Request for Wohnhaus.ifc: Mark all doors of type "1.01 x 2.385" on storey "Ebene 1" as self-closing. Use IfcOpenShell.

First a look at what the model holds.

```python
import ifcopenshell
import ifcopenshell.util.element

model = ifcopenshell.open("Wohnhaus.ifc")
print(model.schema)
storey = next(s for s in model.by_type("IfcBuildingStorey") if s.Name == "Ebene 1")
doors = [e for e in ifcopenshell.util.element.get_decomposition(storey) if e.is_a("IfcDoor")]
seen = {}
for e in doors:
    element_type = ifcopenshell.util.element.get_type(e)
    key = (element_type.Name if element_type != e and element_type else None, ifcopenshell.util.element.get_pset(e, "Pset_DoorCommon", "SelfClosing"))
    seen[key] = seen.get(key, 0) + 1
for (name, value), count in sorted(seen.items(), key=str):
    print(count, "x", name, "|", value)
```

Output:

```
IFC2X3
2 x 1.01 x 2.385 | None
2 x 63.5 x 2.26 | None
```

```python
import ifcopenshell
import ifcopenshell.api.pset
import ifcopenshell.util.element

model = ifcopenshell.open("Wohnhaus.ifc")

storey = next(s for s in model.by_type("IfcBuildingStorey") if s.Name == "Ebene 1")
doors = [e for e in ifcopenshell.util.element.get_decomposition(storey) if e.is_a("IfcDoor")]

count = 0
for e in doors:
    element_type = ifcopenshell.util.element.get_type(e)
    if element_type in (None, e) or element_type.Name != "1.01 x 2.385":
        continue
    # add_pset returns the element's existing set when there is one.
    pset = ifcopenshell.api.pset.add_pset(model, product=e, name="Pset_DoorCommon")
    ifcopenshell.api.pset.edit_pset(model, pset=pset, properties={"SelfClosing": True})
    count += 1

print(count, "doors updated")

model.write("Wohnhaus_updated.ifc")
```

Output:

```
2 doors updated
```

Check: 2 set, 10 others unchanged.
